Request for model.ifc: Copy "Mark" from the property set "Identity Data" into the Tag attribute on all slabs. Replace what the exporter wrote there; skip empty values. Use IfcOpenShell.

First a look at what the model holds.

```python
import ifcopenshell
import ifcopenshell.util.element

model = ifcopenshell.open("model.ifc")
print(model.schema)
slabs = model.by_type("IfcSlab")
print(len(slabs), "slabs")
for e in slabs[:8]:
    source = ifcopenshell.util.element.get_pset(e, "Identity Data", "Mark")
    target = e.Tag
    print(e.id(), repr(source), repr(target), sep=" | ")
```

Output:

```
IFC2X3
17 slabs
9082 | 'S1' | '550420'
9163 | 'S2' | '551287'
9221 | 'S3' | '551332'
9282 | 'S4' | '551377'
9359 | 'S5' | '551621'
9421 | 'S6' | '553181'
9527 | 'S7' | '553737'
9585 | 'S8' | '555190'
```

```python
import ifcopenshell
import ifcopenshell.util.element

model = ifcopenshell.open("model.ifc")

count = 0
for e in model.by_type("IfcSlab"):
    value = ifcopenshell.util.element.get_pset(e, "Identity Data", "Mark")
    current = e.Tag
    if not value or not value.strip() or current == value:
        continue
    e.Tag = value
    count += 1

print(count, "slabs updated")

model.write("model-out.ifc")
```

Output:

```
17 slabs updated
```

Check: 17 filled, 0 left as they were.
